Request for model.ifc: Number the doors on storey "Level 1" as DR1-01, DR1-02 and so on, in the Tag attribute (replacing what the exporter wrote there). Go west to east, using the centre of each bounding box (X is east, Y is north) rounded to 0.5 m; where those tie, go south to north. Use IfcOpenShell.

First a look at what the model holds.

```python
import ifcopenshell
import ifcopenshell.util.element
import ifcopenshell.util.placement

model = ifcopenshell.open("model.ifc")
print(model.schema)
storey = next(s for s in model.by_type("IfcBuildingStorey") if s.Name == "Level 1")
doors = [e for e in ifcopenshell.util.element.get_decomposition(storey) if e.is_a("IfcDoor")]
for e in sorted(doors, key=lambda e: e.id()):
    origin = ifcopenshell.util.placement.get_local_placement(e.ObjectPlacement)[:3, 3]
    print(e.id(), e.Tag, e.Name, origin.round(2) + 0.0, sep=" | ")
```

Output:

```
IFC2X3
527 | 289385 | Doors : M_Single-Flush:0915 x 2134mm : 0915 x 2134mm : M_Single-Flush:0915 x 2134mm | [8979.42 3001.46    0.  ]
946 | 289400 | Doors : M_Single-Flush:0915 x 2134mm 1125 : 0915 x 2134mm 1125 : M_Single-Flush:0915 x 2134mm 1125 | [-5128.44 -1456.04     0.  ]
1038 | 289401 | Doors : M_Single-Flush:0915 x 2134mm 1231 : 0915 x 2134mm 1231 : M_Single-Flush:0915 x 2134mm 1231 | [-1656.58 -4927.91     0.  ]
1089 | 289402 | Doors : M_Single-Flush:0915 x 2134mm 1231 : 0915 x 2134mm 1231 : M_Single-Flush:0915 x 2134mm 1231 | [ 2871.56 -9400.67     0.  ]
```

```python
import ifcopenshell
import ifcopenshell.geom
import ifcopenshell.util.element
import ifcopenshell.util.shape

model = ifcopenshell.open("model.ifc")
settings = ifcopenshell.geom.settings()
settings.set("use-world-coords", True)


def centre(element):
    shape = ifcopenshell.geom.create_shape(settings, element)
    return ifcopenshell.util.shape.get_bbox_centroid(shape.geometry)


storey = next(s for s in model.by_type("IfcBuildingStorey") if s.Name == "Level 1")
doors = [e for e in ifcopenshell.util.element.get_decomposition(storey) if e.is_a("IfcDoor")]

# Insertion points can sit at a corner or the storey origin, so sort by the geometry (in metres).
centres = {e: centre(e) for e in doors}
doors.sort(key=lambda e: (round(centres[e][0] / 0.5), centres[e][1]))

for i, e in enumerate(doors, start=1):
    number = f"DR1-{i:02d}"
    e.Tag = number
    print(e.id(), number)

model.write("model_v2.ifc")
```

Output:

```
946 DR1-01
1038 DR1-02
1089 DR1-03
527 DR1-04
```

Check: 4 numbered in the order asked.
